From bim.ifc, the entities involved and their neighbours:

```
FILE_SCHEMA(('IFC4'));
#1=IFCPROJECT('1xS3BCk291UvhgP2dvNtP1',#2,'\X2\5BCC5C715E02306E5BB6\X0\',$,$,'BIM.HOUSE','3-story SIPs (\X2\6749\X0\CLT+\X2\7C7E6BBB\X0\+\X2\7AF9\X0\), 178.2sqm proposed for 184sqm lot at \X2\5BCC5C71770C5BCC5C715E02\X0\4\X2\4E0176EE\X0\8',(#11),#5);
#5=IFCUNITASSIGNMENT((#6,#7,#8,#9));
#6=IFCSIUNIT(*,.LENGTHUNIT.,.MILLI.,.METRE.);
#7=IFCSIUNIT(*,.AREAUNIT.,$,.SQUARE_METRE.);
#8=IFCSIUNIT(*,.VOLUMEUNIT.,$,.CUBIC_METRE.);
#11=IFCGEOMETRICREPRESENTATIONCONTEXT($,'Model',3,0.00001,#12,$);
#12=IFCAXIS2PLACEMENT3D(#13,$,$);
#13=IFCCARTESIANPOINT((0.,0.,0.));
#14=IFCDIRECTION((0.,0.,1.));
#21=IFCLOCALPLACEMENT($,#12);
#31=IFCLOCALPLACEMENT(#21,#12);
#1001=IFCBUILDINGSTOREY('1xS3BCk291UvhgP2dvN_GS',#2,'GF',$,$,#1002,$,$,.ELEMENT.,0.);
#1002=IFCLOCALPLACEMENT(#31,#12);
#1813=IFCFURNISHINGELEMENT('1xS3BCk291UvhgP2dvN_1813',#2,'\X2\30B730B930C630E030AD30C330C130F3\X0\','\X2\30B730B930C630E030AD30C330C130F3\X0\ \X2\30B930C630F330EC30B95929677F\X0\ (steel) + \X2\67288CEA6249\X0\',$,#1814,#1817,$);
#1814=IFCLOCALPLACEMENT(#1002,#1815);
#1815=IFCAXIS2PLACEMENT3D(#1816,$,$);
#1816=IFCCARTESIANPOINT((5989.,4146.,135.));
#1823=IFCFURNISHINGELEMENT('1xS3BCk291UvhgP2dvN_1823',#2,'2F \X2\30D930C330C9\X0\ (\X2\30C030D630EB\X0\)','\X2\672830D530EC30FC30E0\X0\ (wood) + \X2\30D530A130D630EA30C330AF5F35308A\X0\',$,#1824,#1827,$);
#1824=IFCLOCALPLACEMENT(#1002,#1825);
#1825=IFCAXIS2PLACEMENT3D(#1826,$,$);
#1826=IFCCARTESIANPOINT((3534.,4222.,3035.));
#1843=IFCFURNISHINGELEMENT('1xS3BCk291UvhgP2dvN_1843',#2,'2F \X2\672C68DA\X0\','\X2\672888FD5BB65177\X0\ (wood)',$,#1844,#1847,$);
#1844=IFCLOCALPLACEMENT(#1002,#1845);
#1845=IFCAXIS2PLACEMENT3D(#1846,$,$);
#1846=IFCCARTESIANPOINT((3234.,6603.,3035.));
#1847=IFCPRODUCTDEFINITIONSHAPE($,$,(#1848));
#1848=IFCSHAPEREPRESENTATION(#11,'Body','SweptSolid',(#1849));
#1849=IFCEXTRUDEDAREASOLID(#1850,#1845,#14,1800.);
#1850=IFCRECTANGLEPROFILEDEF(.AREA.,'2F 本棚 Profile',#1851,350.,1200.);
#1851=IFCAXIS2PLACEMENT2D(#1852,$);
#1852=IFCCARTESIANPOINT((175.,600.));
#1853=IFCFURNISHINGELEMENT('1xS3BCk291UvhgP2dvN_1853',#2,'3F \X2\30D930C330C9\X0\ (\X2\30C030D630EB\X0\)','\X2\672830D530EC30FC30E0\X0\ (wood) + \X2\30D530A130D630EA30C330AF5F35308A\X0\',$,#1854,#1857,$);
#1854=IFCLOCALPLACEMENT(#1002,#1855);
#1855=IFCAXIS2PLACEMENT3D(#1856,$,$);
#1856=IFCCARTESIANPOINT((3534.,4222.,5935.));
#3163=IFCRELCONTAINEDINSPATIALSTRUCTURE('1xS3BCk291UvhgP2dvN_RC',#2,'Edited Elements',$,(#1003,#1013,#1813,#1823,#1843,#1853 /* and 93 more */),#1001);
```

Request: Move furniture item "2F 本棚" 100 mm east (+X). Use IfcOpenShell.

```python
import ifcopenshell
import ifcopenshell.api.geometry
import ifcopenshell.util.placement
import ifcopenshell.util.unit

model = ifcopenshell.open("bim.ifc")
unit_scale = ifcopenshell.util.unit.calculate_unit_scale(model)

item = model.by_guid("1xS3BCk291UvhgP2dvN_1843")
matrix = ifcopenshell.util.placement.get_local_placement(item.ObjectPlacement)
matrix[0, 3] += 0.1 / unit_scale
ifcopenshell.api.geometry.edit_object_placement(model, product=item, matrix=matrix, is_si=False)

print(ifcopenshell.util.placement.get_local_placement(item.ObjectPlacement).round(3) + 0.0)

model.write("bim_v2.ifc")
```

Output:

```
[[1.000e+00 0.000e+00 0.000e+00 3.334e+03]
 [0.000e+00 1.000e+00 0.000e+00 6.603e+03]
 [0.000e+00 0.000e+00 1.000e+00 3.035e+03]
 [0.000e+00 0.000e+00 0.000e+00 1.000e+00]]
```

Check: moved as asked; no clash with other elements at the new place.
